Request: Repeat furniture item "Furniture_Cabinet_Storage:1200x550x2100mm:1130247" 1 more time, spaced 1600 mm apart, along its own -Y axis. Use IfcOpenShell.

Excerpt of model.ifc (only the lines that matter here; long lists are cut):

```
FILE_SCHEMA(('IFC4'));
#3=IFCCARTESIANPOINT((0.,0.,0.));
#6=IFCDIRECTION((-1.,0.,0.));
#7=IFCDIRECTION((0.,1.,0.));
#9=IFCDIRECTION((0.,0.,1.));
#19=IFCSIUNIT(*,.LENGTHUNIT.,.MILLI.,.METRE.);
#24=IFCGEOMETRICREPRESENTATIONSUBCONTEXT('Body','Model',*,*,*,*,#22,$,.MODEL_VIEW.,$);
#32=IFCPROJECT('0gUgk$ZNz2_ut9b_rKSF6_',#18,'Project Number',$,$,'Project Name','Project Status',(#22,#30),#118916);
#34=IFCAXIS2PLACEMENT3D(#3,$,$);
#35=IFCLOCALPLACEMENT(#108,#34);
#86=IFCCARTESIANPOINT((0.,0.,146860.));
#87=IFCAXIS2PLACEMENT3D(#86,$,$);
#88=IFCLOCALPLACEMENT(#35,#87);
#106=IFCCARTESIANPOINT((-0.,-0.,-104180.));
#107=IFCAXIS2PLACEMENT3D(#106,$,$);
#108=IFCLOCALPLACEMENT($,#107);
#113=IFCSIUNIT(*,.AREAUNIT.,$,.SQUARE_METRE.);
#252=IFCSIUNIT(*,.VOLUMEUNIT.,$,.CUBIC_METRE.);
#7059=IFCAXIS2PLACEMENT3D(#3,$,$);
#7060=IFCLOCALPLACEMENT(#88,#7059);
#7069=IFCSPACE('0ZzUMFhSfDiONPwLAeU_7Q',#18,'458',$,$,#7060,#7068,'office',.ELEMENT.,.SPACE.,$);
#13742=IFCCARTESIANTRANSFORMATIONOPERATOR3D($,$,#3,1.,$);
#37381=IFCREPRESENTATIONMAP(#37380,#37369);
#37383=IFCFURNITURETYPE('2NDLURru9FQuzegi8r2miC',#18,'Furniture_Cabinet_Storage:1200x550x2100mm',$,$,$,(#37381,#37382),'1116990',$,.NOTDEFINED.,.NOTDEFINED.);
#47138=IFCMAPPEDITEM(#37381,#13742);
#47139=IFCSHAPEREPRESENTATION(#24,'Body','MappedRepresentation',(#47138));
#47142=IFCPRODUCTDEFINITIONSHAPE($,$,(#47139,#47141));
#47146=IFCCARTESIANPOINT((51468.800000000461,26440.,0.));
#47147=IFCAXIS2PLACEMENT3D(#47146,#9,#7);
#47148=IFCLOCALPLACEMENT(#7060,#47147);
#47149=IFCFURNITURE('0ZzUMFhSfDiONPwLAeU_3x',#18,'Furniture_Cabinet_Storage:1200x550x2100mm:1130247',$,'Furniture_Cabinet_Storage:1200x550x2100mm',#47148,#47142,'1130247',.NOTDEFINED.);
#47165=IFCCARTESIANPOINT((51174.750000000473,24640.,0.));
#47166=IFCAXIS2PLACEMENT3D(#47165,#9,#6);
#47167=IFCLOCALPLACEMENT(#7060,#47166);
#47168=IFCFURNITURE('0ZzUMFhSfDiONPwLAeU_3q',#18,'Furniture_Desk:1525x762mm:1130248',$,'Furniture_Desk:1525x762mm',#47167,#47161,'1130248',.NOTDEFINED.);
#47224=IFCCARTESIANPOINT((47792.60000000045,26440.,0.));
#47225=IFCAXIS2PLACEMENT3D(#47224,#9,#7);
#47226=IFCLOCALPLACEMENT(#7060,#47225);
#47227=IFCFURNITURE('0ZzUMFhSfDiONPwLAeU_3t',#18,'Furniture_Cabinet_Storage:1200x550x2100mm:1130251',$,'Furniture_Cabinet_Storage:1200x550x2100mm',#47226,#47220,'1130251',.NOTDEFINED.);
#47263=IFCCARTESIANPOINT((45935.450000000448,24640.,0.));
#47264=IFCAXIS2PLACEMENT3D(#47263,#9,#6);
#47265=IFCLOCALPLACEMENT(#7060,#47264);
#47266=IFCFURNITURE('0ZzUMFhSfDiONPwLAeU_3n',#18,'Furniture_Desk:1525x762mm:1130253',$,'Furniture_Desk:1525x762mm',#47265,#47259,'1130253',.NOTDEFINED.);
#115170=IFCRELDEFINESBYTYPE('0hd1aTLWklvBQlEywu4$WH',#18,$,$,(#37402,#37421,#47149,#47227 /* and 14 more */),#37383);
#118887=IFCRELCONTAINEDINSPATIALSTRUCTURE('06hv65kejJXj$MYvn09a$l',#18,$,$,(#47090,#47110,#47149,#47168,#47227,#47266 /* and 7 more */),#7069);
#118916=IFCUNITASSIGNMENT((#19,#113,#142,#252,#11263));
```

```python
import ifcopenshell
import ifcopenshell.api.geometry
import ifcopenshell.api.root
import ifcopenshell.util.element
import ifcopenshell.util.placement

model = ifcopenshell.open("model.ifc")


def reuse_history(source, copy):
    """copy_class also copies each property set's owner history, people and application; keep the originals."""
    for rel in copy.IsDefinedBy:
        if rel.is_a("IfcRelDefinesByProperties") and (history := rel.RelatingPropertyDefinition.OwnerHistory):
            rel.RelatingPropertyDefinition.OwnerHistory = source.OwnerHistory
            ifcopenshell.util.element.remove_deep2(model, history)


source = model.by_guid("0ZzUMFhSfDiONPwLAeU_3x")
base = ifcopenshell.util.placement.get_local_placement(source.ObjectPlacement)
step = -base[:3, 1] * 1600.0

for i in range(1, 2):
    copy = ifcopenshell.api.root.copy_class(model, product=source)
    copy.Representation = ifcopenshell.util.element.copy_deep(
        model, source.Representation, exclude=["IfcGeometricRepresentationContext", "IfcRepresentationMap"]
    )
    copy.Name = "Furniture_Cabinet_Storage:1200x550x2100mm"
    copy.Tag = None
    reuse_history(source, copy)
    matrix = base.copy()
    matrix[:3, 3] += i * step
    print("added at", matrix[:3, 3].round(3) + 0.0)
    ifcopenshell.api.geometry.edit_object_placement(model, product=copy, matrix=matrix, is_si=False)

model.write("model_v2.ifc")
```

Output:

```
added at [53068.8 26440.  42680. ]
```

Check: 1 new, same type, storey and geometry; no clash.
